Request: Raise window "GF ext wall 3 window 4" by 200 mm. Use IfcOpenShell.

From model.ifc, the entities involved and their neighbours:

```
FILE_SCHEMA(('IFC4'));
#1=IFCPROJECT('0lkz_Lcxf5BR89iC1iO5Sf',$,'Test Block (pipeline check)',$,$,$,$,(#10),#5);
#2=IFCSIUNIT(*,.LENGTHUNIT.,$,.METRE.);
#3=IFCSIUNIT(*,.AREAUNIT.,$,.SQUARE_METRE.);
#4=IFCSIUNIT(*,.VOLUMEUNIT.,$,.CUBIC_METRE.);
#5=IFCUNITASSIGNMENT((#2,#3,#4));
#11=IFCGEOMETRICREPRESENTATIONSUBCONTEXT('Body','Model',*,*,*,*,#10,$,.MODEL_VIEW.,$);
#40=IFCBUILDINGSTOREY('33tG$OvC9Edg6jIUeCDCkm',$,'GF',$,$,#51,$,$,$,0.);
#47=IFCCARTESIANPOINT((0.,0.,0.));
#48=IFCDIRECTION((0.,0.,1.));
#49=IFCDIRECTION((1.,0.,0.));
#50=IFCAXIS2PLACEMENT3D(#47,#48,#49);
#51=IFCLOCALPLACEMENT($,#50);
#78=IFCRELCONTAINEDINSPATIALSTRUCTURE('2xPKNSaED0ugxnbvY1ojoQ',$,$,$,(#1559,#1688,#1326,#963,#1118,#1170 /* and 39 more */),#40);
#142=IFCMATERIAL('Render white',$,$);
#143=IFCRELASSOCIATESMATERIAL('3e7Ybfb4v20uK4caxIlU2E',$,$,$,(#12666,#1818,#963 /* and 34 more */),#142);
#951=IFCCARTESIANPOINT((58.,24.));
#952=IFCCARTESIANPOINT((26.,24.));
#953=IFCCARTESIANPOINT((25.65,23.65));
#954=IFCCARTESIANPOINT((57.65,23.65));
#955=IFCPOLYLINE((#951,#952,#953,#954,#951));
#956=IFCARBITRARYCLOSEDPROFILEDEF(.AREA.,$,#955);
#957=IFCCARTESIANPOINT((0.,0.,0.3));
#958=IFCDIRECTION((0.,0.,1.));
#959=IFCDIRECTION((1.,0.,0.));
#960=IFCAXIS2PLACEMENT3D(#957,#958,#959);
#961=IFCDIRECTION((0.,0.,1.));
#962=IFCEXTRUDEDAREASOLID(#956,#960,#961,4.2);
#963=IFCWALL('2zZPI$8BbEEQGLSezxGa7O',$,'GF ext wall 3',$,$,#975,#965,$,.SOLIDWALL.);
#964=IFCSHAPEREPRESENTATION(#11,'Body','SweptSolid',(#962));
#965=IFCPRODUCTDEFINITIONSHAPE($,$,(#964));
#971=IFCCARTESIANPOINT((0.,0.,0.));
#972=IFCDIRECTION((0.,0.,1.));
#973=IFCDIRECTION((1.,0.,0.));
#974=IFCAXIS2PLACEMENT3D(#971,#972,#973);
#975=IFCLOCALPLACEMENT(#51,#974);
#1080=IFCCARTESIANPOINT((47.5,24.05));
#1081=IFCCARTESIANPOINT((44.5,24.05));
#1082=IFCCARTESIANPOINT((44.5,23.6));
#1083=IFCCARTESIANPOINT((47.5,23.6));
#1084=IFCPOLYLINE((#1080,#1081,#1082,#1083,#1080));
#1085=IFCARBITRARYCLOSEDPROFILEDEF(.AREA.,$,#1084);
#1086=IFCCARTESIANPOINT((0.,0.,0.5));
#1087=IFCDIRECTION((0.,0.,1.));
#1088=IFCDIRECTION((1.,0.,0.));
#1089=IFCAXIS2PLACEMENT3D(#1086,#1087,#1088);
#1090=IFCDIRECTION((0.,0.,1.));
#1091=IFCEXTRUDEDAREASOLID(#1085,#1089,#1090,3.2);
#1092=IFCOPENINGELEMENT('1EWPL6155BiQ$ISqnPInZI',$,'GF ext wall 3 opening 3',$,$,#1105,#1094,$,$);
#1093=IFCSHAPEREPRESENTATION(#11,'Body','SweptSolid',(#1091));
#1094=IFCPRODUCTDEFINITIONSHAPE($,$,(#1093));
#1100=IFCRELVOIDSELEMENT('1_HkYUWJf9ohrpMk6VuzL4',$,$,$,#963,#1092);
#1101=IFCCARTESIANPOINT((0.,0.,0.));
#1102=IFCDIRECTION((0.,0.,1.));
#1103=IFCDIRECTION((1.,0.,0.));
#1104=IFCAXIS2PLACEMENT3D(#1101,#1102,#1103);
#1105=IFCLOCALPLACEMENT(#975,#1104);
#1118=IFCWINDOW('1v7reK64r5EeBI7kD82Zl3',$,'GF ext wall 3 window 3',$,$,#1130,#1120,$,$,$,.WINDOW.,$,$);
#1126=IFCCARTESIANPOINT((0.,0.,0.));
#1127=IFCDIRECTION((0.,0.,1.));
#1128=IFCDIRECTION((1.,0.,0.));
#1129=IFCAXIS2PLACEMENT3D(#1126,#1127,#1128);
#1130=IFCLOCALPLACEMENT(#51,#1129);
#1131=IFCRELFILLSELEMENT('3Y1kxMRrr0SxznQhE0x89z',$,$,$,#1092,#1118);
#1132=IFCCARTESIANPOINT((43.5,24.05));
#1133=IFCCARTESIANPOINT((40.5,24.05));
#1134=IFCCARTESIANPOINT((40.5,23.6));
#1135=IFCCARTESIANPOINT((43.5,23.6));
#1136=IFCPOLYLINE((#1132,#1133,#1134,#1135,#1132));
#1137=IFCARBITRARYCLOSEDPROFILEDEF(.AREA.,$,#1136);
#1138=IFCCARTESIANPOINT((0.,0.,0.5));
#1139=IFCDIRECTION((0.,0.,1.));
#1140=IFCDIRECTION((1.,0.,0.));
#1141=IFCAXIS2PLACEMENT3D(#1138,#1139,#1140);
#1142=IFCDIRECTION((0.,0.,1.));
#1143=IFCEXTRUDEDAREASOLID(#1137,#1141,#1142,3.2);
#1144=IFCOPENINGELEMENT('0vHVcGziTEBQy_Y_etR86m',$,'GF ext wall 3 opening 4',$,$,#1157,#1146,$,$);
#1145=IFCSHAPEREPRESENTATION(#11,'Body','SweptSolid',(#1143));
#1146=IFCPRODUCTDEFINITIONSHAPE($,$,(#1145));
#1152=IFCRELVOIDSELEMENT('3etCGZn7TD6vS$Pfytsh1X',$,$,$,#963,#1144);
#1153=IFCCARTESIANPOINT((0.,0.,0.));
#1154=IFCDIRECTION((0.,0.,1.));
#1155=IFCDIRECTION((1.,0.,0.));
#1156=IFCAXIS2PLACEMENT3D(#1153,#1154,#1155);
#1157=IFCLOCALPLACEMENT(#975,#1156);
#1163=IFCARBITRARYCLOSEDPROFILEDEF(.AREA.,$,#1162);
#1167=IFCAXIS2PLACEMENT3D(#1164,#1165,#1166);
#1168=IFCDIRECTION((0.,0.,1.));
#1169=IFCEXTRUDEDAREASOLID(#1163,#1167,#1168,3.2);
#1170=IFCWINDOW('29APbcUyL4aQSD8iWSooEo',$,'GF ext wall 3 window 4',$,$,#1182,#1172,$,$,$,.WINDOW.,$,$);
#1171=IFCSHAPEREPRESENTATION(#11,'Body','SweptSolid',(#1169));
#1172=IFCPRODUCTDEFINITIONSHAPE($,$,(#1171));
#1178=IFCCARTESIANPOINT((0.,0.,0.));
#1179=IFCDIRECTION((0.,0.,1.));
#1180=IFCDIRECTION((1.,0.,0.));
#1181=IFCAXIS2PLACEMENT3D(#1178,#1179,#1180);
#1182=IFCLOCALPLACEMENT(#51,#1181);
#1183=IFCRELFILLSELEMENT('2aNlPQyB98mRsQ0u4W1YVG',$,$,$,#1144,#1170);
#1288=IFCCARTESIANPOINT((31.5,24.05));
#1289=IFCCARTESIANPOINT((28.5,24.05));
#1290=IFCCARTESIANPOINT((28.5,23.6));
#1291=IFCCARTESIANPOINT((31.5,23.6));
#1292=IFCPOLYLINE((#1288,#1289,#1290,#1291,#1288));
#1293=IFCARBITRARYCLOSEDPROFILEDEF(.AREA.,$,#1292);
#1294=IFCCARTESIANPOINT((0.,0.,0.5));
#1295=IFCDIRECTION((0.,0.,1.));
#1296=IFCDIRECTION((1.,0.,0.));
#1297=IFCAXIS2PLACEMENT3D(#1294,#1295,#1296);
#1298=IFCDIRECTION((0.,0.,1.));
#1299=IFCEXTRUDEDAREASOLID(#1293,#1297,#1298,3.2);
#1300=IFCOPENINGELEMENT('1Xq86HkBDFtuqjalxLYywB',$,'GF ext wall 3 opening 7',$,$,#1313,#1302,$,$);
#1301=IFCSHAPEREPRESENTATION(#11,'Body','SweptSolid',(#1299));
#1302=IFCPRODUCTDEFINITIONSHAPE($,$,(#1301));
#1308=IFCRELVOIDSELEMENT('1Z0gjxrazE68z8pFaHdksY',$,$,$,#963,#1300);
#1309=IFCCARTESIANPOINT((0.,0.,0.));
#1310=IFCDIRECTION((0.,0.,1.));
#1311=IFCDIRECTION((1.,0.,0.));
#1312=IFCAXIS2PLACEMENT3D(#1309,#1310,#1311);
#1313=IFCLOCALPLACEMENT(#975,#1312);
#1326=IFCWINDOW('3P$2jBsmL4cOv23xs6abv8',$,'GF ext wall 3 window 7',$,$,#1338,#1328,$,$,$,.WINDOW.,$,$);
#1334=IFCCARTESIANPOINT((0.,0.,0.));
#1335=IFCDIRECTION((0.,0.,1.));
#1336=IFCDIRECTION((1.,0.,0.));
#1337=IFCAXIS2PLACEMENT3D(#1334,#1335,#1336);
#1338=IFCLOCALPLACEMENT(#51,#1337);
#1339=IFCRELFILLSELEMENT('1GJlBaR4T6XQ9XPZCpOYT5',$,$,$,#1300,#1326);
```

```python
import numpy as np
import ifcopenshell
import ifcopenshell.api.geometry
import ifcopenshell.util.placement
import ifcopenshell.util.unit

model = ifcopenshell.open("model.ifc")
unit_scale = ifcopenshell.util.unit.calculate_unit_scale(model)

window = model.by_guid("29APbcUyL4aQSD8iWSooEo")
opening = window.FillsVoids[0].RelatingOpeningElement
dz = 0.2 / unit_scale

shift = np.array([0.0, 0.0, dz])
# The window is not placed relative to its opening, so move both.
for product in (opening, window):
    matrix = ifcopenshell.util.placement.get_local_placement(product.ObjectPlacement)
    matrix[:3, 3] += shift
    ifcopenshell.api.geometry.edit_object_placement(model, product=product, matrix=matrix, is_si=False)

print(f"moved by {dz * unit_scale:+.3f} m")

model.write("model_v2.ifc")
```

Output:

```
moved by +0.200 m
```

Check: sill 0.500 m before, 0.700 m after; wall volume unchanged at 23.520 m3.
